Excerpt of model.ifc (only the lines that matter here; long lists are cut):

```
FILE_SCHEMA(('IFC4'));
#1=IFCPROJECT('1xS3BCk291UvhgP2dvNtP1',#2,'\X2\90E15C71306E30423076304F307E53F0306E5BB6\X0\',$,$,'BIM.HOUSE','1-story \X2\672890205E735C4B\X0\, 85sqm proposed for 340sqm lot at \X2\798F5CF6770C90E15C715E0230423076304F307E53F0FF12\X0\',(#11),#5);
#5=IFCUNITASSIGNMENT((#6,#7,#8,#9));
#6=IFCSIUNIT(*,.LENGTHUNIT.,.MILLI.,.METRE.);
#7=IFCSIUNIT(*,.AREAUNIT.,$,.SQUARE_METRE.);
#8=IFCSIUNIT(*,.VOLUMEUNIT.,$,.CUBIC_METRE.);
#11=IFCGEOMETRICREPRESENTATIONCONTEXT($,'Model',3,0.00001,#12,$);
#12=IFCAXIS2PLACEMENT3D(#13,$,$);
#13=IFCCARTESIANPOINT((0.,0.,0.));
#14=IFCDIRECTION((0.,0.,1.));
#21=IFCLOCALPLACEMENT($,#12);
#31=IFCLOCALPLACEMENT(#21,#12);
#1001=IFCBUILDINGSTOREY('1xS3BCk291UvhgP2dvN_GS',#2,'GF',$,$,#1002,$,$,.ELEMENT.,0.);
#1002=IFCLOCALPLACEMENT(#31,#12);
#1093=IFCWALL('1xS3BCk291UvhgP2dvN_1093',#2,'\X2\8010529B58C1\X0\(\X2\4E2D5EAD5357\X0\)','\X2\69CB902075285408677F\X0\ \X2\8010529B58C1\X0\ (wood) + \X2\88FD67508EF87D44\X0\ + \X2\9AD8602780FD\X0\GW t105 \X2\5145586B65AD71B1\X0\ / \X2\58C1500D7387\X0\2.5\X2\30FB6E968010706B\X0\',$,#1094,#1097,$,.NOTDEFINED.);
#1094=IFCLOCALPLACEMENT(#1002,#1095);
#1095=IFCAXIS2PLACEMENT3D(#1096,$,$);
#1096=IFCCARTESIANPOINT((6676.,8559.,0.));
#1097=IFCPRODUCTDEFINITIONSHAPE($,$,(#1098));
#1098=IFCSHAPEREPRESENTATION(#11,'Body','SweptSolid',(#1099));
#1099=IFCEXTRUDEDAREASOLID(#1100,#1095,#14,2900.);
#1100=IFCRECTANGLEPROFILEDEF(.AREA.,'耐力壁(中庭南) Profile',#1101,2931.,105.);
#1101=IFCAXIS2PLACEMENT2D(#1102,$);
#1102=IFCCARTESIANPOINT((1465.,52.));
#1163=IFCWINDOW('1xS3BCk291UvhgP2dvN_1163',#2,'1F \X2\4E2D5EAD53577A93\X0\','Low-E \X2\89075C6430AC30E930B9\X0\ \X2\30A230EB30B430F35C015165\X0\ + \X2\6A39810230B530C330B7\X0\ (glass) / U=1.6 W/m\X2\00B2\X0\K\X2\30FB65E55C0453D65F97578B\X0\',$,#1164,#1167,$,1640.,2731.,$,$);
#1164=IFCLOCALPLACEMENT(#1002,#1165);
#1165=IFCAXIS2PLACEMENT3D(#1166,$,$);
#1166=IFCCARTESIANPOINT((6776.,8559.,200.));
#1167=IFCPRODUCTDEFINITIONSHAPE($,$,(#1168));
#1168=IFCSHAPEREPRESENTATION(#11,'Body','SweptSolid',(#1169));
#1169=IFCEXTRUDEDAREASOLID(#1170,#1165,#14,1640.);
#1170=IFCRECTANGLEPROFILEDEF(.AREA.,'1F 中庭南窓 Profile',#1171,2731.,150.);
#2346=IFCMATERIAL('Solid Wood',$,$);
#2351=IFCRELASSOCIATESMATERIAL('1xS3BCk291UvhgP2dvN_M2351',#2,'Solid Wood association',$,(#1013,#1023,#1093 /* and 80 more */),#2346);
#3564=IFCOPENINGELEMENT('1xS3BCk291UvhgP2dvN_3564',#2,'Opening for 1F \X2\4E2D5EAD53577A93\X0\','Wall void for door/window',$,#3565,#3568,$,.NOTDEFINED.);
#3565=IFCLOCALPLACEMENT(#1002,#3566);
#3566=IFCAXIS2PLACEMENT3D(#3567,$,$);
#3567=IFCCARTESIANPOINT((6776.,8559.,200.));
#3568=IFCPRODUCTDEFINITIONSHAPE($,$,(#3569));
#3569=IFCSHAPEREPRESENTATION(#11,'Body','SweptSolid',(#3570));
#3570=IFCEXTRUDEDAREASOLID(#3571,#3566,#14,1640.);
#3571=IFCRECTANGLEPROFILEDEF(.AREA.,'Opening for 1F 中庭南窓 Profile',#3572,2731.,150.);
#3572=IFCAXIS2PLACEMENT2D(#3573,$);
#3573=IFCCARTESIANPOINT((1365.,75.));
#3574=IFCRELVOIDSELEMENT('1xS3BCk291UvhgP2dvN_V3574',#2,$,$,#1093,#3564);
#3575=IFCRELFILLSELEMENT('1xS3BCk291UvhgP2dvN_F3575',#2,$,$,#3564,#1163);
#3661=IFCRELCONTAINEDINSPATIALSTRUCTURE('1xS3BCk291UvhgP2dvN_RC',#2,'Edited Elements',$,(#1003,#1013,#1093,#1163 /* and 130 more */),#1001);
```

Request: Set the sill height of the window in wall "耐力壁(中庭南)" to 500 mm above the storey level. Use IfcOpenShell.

```python
import numpy as np
import ifcopenshell
import ifcopenshell.api.geometry
import ifcopenshell.geom
import ifcopenshell.util.element
import ifcopenshell.util.placement
import ifcopenshell.util.shape
import ifcopenshell.util.unit

model = ifcopenshell.open("model.ifc")
unit_scale = ifcopenshell.util.unit.calculate_unit_scale(model)

window = model.by_guid("1xS3BCk291UvhgP2dvN_1163")
opening = window.FillsVoids[0].RelatingOpeningElement
storey = ifcopenshell.util.element.get_container(window, ifc_class="IfcBuildingStorey")
level = ifcopenshell.util.placement.get_local_placement(storey.ObjectPlacement)[2, 3]

# The opening's origin need not be at the sill, so measure its lowest point.
shape = ifcopenshell.geom.create_shape(ifcopenshell.geom.settings(), opening)
bottom = ifcopenshell.util.shape.get_shape_bottom_elevation(shape, shape.geometry) / unit_scale
dz = level + 500.0 - bottom

shift = np.array([0.0, 0.0, dz])
# The window is not placed relative to its opening, so move both.
for product in (opening, window):
    matrix = ifcopenshell.util.placement.get_local_placement(product.ObjectPlacement)
    matrix[:3, 3] += shift
    ifcopenshell.api.geometry.edit_object_placement(model, product=product, matrix=matrix, is_si=False)

print(f"moved by {dz * unit_scale:+.3f} m")

model.write("model_edited.ifc")
```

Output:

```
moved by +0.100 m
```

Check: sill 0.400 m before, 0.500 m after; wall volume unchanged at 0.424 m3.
